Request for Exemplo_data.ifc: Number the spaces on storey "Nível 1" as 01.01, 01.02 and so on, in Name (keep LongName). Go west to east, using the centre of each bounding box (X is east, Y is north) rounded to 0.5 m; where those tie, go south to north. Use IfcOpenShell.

First a look at what the model holds.

```python
import ifcopenshell
import ifcopenshell.util.element
import ifcopenshell.util.placement

model = ifcopenshell.open("Exemplo_data.ifc")
print(model.schema)
storey = next(s for s in model.by_type("IfcBuildingStorey") if s.Name == "Nível 1")
spaces = [e for e in ifcopenshell.util.element.get_decomposition(storey) if e.is_a("IfcSpace")]
for e in sorted(spaces, key=lambda e: e.id()):
    origin = ifcopenshell.util.placement.get_local_placement(e.ObjectPlacement)[:3, 3]
    print(e.id(), e.Name, e.LongName, origin.round(2) + 0.0, sep=" | ")
```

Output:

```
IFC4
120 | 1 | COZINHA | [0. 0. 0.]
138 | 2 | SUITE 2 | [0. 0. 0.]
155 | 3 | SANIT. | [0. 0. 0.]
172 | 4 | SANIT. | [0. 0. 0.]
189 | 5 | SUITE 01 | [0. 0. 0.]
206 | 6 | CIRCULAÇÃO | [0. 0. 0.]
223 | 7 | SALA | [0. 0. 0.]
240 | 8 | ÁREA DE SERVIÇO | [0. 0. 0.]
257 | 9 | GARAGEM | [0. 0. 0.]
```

```python
import ifcopenshell
import ifcopenshell.geom
import ifcopenshell.util.element
import ifcopenshell.util.shape

model = ifcopenshell.open("Exemplo_data.ifc")
settings = ifcopenshell.geom.settings()
settings.set("use-world-coords", True)


def centre(element):
    shape = ifcopenshell.geom.create_shape(settings, element)
    return ifcopenshell.util.shape.get_bbox_centroid(shape.geometry)


storey = next(s for s in model.by_type("IfcBuildingStorey") if s.Name == "Nível 1")
spaces = [e for e in ifcopenshell.util.element.get_decomposition(storey) if e.is_a("IfcSpace")]

# Insertion points can sit at a corner or the storey origin, so sort by the geometry (in metres).
centres = {e: centre(e) for e in spaces}
spaces.sort(key=lambda e: (round(centres[e][0] / 0.5), centres[e][1]))

for i, e in enumerate(spaces, start=1):
    number = f"01.{i:02d}"
    e.Name = number
    print(e.id(), number)

model.write("Exemplo_data_updated.ifc")
```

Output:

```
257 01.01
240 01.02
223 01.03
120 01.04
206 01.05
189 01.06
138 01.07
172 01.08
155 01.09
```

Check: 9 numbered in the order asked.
